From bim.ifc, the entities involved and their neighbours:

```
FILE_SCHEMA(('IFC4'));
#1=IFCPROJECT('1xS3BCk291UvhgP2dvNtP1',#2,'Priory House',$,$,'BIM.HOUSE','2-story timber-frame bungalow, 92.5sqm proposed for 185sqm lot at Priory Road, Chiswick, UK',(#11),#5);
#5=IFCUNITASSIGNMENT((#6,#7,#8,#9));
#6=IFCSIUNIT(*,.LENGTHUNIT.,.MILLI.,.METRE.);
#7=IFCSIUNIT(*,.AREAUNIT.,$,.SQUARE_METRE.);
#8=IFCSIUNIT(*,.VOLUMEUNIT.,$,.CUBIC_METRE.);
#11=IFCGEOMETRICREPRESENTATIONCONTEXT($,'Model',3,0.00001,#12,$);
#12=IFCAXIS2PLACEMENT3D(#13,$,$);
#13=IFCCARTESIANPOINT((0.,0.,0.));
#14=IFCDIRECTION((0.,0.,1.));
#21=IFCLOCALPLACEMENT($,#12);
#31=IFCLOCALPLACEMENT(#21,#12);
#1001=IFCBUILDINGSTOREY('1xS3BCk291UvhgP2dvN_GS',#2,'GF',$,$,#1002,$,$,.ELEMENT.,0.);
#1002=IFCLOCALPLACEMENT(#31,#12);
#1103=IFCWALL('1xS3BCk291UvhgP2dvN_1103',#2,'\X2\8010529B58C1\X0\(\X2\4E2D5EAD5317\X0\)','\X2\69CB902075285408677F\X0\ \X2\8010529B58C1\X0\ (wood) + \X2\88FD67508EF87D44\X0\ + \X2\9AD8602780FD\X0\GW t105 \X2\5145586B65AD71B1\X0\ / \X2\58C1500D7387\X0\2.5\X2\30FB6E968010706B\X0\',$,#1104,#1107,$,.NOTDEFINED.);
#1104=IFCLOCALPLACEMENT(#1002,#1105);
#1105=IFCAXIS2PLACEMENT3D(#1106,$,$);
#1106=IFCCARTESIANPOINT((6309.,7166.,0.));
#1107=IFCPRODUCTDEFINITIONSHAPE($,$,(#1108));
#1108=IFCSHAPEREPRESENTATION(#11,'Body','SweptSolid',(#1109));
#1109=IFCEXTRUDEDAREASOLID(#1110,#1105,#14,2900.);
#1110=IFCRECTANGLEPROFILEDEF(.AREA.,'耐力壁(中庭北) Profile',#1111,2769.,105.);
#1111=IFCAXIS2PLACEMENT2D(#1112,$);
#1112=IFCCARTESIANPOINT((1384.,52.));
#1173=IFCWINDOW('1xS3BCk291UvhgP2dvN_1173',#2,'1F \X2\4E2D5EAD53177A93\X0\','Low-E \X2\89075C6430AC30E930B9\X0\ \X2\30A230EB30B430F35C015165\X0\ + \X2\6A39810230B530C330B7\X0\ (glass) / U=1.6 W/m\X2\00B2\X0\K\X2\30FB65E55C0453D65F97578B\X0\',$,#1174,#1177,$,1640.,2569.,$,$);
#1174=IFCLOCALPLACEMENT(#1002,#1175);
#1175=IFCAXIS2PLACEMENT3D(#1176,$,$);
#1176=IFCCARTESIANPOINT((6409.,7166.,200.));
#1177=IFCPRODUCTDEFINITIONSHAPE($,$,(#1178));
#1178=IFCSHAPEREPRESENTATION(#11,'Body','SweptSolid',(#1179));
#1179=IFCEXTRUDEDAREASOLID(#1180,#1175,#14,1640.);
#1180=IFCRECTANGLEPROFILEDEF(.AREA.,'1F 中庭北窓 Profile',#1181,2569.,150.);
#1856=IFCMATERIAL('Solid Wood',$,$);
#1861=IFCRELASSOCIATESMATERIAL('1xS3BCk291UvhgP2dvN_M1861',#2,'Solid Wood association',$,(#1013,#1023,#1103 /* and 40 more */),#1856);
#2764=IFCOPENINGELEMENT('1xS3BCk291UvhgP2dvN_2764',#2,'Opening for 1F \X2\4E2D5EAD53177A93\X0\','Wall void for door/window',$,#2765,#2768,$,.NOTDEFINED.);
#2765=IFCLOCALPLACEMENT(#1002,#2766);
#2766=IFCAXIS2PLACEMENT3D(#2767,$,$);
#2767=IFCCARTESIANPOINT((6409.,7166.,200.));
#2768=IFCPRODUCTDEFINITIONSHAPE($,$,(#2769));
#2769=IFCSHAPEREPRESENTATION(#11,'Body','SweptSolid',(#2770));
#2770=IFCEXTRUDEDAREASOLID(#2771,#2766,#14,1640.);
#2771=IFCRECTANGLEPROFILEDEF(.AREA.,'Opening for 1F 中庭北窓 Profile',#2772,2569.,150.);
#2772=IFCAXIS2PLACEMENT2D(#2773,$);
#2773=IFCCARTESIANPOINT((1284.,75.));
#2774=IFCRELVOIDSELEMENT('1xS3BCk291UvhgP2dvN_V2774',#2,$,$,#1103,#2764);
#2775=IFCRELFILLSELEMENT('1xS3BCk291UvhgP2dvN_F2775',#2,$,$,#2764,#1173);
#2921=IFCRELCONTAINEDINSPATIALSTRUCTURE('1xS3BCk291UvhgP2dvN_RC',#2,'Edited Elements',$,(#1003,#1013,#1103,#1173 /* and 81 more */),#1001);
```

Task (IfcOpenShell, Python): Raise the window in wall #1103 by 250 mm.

```python
import numpy as np
import ifcopenshell
import ifcopenshell.api.geometry
import ifcopenshell.util.placement
import ifcopenshell.util.unit

model = ifcopenshell.open("bim.ifc")
unit_scale = ifcopenshell.util.unit.calculate_unit_scale(model)

window = model.by_guid("1xS3BCk291UvhgP2dvN_1173")
opening = window.FillsVoids[0].RelatingOpeningElement
dz = 0.25 / unit_scale

shift = np.array([0.0, 0.0, dz])
# The window is not placed relative to its opening, so move both.
for product in (opening, window):
    matrix = ifcopenshell.util.placement.get_local_placement(product.ObjectPlacement)
    matrix[:3, 3] += shift
    ifcopenshell.api.geometry.edit_object_placement(model, product=product, matrix=matrix, is_si=False)

print(f"moved by {dz * unit_scale:+.3f} m")

model.write("bim_edited.ifc")
```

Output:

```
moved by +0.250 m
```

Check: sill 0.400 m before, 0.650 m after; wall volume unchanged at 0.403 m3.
